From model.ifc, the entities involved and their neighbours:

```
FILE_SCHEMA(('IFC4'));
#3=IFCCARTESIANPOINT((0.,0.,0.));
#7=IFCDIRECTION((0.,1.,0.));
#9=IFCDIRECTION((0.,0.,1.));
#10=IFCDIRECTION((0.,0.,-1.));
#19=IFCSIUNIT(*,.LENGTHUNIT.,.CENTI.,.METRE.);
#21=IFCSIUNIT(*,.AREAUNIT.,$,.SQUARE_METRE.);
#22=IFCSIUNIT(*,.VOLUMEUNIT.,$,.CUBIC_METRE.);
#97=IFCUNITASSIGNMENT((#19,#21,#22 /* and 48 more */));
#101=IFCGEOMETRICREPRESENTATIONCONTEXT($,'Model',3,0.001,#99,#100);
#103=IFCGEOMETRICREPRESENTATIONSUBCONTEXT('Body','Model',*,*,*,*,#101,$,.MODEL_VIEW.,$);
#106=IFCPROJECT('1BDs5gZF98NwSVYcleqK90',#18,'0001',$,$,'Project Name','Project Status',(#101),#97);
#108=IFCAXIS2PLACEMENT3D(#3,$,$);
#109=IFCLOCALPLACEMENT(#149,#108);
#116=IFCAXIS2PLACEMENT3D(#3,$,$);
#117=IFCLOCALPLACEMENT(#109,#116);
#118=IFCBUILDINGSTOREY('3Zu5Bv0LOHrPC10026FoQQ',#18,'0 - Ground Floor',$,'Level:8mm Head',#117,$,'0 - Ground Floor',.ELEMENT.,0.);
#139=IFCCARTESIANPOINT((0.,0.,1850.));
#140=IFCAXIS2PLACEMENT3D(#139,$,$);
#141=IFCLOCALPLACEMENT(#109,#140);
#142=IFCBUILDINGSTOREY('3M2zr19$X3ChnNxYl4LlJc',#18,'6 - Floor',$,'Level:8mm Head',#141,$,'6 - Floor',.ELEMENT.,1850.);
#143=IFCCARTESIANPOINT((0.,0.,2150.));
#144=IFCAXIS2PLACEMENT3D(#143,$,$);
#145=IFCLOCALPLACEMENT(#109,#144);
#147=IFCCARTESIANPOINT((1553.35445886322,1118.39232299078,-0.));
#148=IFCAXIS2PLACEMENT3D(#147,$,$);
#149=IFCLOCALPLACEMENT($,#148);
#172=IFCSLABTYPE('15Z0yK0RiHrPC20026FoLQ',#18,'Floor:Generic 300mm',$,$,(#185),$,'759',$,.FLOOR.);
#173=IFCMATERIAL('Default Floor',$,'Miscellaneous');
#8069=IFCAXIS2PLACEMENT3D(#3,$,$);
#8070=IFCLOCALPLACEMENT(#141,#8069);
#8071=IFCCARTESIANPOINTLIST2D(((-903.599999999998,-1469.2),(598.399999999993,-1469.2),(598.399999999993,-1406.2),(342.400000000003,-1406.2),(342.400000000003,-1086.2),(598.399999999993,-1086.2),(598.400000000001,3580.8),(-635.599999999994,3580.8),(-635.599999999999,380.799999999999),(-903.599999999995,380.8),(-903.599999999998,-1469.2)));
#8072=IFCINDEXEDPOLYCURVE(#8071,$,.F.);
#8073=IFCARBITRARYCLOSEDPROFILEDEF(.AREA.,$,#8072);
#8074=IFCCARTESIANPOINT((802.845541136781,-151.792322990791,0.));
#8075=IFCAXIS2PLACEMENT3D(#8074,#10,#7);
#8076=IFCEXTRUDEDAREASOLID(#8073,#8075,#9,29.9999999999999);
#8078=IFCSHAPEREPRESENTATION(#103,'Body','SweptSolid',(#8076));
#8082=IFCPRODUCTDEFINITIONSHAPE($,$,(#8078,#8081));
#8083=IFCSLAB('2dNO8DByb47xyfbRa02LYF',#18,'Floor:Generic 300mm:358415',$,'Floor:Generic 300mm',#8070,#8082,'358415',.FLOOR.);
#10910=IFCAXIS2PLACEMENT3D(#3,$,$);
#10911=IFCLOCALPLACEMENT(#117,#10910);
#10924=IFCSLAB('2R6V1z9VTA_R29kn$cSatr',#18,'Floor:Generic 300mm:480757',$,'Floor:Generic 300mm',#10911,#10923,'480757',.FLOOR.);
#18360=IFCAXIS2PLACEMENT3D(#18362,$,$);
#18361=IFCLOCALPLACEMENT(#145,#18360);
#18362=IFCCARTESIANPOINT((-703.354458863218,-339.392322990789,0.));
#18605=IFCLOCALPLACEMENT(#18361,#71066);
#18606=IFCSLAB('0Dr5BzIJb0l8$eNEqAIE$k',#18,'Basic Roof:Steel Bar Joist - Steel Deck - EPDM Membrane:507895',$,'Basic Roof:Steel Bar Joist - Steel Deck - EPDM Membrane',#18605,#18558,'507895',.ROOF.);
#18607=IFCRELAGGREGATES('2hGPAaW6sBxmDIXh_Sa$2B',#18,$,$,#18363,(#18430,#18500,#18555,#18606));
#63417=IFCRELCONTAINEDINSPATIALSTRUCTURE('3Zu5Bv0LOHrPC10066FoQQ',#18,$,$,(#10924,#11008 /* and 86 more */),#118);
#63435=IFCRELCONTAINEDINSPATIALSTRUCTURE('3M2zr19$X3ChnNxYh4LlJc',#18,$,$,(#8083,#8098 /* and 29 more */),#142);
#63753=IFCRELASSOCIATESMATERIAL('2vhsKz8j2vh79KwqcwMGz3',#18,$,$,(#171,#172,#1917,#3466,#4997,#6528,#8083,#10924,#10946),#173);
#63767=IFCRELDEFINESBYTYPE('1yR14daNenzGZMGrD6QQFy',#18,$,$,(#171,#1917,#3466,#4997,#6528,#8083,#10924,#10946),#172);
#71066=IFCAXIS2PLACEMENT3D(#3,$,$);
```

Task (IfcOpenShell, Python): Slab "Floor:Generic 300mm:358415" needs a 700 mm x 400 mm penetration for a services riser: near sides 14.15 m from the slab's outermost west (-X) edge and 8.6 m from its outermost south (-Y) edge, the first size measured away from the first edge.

```python
import numpy as np
import ifcopenshell
import ifcopenshell.api.feature
import ifcopenshell.api.geometry
import ifcopenshell.api.root
import ifcopenshell.geom
import ifcopenshell.util.placement
import ifcopenshell.util.representation
import ifcopenshell.util.shape
import ifcopenshell.util.unit

model = ifcopenshell.open("model.ifc")
unit_scale = ifcopenshell.util.unit.calculate_unit_scale(model)
settings = ifcopenshell.geom.settings()


def volume(element):
    """Net volume in cubic metres, openings subtracted."""
    shape = ifcopenshell.geom.create_shape(settings, element)
    return ifcopenshell.util.shape.get_volume(shape.geometry)


slab = model.by_id(8083)
before = volume(slab)

# Extent in the slab's own axes, in metres. The edges named are its -X and -Y sides.
slab_shape = ifcopenshell.geom.create_shape(settings, slab)
vertices = ifcopenshell.util.shape.get_vertices(slab_shape.geometry)
x_min, y_min, bottom = vertices.min(axis=0)
top = vertices[:, 2].max()

opening = ifcopenshell.api.root.create_entity(model, ifc_class="IfcOpeningElement", name="Services riser opening", predefined_type="OPENING")
context = ifcopenshell.util.representation.get_context(model, "Model", "Body", "MODEL_VIEW")
width, depth = 0.7, 0.4
outline = [(0.0, 0.0), (width, 0.0), (width, depth), (0.0, depth), (0.0, 0.0)]
# Overshoot both faces by 50 mm so the cut is clean.
shape = ifcopenshell.api.geometry.add_slab_representation(
    model, context=context, depth=top - bottom + 0.1, polyline=outline
)
ifcopenshell.api.geometry.assign_representation(model, product=opening, representation=shape)

matrix = ifcopenshell.util.placement.get_local_placement(slab.ObjectPlacement)
matrix[:, 3] = matrix @ np.append(np.array([x_min + 14.15, y_min + 8.6, bottom - 0.05]) / unit_scale, 1.0)
ifcopenshell.api.geometry.edit_object_placement(model, product=opening, matrix=matrix, is_si=False)
ifcopenshell.api.feature.add_feature(model, feature=opening, element=slab)

after = volume(slab)

print(f"slab volume {before:.3f} -> {after:.3f} m3")

model.write("model_rev.ifc")
```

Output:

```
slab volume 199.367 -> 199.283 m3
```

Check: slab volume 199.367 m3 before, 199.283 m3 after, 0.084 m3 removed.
